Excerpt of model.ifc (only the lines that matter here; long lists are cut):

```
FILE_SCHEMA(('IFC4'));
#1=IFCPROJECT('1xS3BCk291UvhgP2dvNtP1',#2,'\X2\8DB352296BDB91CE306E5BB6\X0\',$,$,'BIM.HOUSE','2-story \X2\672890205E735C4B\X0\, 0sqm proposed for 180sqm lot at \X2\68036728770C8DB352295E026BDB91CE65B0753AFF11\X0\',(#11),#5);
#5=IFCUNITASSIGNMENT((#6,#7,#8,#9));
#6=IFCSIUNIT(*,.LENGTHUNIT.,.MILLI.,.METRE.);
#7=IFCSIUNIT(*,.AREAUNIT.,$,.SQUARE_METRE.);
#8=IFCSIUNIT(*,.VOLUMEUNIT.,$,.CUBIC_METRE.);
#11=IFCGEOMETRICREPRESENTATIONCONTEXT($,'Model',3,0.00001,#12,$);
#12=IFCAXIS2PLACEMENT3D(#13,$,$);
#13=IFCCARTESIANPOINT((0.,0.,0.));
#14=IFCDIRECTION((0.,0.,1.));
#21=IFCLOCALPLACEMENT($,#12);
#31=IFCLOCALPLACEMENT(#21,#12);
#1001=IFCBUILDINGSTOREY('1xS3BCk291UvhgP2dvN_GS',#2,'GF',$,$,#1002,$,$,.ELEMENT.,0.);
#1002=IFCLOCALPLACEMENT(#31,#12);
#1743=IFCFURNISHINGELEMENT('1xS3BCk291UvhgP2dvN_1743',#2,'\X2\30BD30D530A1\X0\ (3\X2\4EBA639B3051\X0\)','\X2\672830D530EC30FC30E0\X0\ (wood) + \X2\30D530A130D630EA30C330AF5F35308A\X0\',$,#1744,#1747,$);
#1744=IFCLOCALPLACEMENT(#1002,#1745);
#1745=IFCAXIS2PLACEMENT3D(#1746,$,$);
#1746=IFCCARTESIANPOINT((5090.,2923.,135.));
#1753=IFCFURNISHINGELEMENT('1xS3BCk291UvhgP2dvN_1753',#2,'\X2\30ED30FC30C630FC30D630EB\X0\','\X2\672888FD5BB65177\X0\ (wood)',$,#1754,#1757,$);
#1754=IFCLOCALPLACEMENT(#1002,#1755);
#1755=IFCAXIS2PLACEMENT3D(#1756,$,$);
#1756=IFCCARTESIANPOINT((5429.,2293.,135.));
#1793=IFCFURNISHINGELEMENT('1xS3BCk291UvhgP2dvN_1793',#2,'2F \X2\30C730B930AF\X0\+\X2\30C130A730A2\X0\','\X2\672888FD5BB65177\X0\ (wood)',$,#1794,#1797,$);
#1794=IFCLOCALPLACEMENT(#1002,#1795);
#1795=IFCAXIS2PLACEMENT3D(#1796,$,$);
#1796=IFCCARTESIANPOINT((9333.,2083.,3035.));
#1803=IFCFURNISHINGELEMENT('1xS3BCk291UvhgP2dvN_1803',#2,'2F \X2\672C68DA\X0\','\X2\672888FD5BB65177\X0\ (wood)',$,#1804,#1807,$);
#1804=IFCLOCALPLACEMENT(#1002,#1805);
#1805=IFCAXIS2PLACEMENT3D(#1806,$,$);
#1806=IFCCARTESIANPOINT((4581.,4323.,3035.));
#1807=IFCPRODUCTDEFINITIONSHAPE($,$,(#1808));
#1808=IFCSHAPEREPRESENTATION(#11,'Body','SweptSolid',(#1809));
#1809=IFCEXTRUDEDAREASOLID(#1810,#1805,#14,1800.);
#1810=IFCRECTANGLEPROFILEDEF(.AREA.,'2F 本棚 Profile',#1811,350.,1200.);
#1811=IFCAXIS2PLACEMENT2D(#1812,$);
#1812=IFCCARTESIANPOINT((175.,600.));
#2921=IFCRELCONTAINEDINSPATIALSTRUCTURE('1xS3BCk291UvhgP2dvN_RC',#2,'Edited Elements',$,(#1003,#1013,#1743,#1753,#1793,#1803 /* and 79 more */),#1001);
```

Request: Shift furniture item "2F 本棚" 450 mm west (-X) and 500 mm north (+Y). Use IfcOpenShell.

```python
import ifcopenshell
import ifcopenshell.api.geometry
import ifcopenshell.util.placement
import ifcopenshell.util.unit

model = ifcopenshell.open("model.ifc")
unit_scale = ifcopenshell.util.unit.calculate_unit_scale(model)

item = model.by_guid("1xS3BCk291UvhgP2dvN_1803")
matrix = ifcopenshell.util.placement.get_local_placement(item.ObjectPlacement)
matrix[0, 3] -= 0.45 / unit_scale
matrix[1, 3] += 0.5 / unit_scale
ifcopenshell.api.geometry.edit_object_placement(model, product=item, matrix=matrix, is_si=False)

print(ifcopenshell.util.placement.get_local_placement(item.ObjectPlacement).round(3) + 0.0)

model.write("model_v2.ifc")
```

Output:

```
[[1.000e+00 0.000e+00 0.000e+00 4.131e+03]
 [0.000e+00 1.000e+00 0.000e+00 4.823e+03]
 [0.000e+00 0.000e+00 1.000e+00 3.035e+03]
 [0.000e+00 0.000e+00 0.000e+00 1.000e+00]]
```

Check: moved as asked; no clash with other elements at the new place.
